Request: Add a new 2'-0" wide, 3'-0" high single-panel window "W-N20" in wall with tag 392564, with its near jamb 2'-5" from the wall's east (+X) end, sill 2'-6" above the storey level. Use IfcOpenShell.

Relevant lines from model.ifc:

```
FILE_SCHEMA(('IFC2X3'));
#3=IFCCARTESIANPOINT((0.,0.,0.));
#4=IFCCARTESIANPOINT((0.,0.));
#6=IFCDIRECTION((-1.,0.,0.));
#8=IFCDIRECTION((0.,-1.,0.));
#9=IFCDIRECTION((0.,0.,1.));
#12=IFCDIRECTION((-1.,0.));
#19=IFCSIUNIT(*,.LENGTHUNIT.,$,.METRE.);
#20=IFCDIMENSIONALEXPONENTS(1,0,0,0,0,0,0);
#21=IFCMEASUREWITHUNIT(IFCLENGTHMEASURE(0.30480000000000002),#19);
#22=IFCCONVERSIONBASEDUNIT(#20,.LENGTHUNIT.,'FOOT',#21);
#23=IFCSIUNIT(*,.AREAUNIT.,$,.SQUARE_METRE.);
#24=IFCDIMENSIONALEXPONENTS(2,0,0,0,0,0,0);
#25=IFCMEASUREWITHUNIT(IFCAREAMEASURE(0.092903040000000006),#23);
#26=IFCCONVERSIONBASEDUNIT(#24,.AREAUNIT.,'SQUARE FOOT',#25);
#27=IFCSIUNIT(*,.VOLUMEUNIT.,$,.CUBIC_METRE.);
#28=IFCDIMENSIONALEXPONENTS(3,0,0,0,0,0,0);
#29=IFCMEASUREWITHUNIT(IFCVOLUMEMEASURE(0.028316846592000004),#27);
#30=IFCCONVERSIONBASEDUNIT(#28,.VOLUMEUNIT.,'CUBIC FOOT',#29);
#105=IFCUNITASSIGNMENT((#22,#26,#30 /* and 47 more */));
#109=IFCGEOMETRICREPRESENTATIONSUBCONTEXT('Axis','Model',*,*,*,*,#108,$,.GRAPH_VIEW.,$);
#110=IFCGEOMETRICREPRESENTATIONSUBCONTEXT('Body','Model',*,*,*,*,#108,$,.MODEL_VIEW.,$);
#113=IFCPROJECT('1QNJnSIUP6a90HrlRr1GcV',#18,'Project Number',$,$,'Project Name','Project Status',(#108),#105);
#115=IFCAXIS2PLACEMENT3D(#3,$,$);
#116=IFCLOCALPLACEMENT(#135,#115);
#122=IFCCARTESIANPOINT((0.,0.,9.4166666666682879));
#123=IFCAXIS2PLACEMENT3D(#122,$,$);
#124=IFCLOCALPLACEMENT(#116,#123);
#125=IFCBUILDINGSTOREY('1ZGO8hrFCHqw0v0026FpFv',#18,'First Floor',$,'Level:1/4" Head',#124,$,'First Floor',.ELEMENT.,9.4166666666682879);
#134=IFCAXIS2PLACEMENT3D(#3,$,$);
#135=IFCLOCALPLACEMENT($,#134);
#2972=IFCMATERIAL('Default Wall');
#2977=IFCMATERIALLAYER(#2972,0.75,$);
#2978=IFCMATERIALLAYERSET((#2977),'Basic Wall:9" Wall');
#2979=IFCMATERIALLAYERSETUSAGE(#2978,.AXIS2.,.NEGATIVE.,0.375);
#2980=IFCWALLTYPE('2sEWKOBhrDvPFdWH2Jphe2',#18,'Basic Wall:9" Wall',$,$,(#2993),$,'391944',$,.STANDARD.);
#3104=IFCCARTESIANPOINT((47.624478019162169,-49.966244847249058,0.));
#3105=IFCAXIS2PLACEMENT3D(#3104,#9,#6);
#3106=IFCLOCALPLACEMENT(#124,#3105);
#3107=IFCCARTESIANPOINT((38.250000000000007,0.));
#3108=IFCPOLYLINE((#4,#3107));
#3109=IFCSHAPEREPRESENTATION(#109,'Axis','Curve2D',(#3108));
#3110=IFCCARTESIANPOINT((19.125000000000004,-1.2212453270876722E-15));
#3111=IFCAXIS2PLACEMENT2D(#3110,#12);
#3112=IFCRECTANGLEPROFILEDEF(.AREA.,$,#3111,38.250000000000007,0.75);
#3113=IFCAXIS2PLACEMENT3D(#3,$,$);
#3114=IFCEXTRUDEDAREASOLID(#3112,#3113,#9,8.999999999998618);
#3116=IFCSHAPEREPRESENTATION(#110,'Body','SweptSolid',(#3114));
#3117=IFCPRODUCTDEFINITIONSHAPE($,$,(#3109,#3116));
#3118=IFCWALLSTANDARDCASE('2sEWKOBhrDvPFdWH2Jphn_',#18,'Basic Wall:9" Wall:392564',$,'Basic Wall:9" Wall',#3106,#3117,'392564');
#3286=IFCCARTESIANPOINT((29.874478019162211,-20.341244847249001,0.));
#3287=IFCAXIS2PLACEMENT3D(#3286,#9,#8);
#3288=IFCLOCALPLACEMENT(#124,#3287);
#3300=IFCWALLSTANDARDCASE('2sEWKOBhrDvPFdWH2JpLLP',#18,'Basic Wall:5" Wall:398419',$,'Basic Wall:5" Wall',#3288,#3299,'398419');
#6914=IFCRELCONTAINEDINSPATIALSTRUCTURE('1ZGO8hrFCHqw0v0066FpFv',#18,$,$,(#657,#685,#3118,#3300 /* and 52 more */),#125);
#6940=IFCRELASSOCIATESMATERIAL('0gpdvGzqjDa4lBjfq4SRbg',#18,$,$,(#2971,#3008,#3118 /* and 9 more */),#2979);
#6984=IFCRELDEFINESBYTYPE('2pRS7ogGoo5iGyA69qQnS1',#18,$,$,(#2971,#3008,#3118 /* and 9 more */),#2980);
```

```python
import numpy as np
import ifcopenshell
import ifcopenshell.api.feature
import ifcopenshell.api.geometry
import ifcopenshell.api.root
import ifcopenshell.api.spatial
import ifcopenshell.api.type
import ifcopenshell.geom
import ifcopenshell.util.element
import ifcopenshell.util.placement
import ifcopenshell.util.representation
import ifcopenshell.util.shape
import ifcopenshell.util.unit

model = ifcopenshell.open("model.ifc")
unit_scale = ifcopenshell.util.unit.calculate_unit_scale(model)
settings = ifcopenshell.geom.settings()


def volume(element):
    """Net volume in cubic metres, openings subtracted."""
    shape = ifcopenshell.geom.create_shape(settings, element)
    return ifcopenshell.util.shape.get_volume(shape.geometry)


wall = model.by_id(3118)
storey = ifcopenshell.util.element.get_container(wall, ifc_class="IfcBuildingStorey")
context = ifcopenshell.util.representation.get_context(model, "Model", "Body", "MODEL_VIEW")
before = volume(wall)

width, height, from_end, sill = 0.6096, 0.9144, 0.7366, 0.762  # metres

# The wall runs along its own X axis, and the end named is its -X end.
wall_shape = ifcopenshell.geom.create_shape(settings, wall)
x, y, z = ifcopenshell.util.shape.get_vertices(wall_shape.geometry).T
start = x.min() + from_end
face, thickness = float(y.min()), float(y.max() - y.min())
wall_matrix = ifcopenshell.util.placement.get_local_placement(wall.ObjectPlacement)
level = ifcopenshell.util.placement.get_local_placement(storey.ObjectPlacement)[2, 3]


def in_wall(x, y):
    """Placement at x, y metres in the wall's axes, at sill height."""
    matrix = wall_matrix.copy()
    matrix[:, 3] = wall_matrix @ np.array([x / unit_scale, y / unit_scale, 0.0, 1.0])
    matrix[2, 3] = level + sill / unit_scale
    return matrix


# Opening: a box that overshoots both wall faces by 50 mm.
opening = ifcopenshell.api.root.create_entity(model, ifc_class="IfcOpeningElement")
box = ifcopenshell.api.geometry.add_wall_representation(
    model, context=context, length=width, height=height, thickness=thickness + 0.1
)
ifcopenshell.api.geometry.assign_representation(model, product=opening, representation=box)
ifcopenshell.api.geometry.edit_object_placement(model, product=opening, matrix=in_wall(start, face - 0.05), is_si=False)
ifcopenshell.api.feature.add_feature(model, feature=opening, element=wall)

window = ifcopenshell.api.root.create_entity(model, ifc_class="IfcWindow", name="W-N20")
window.OverallWidth, window.OverallHeight = width / unit_scale, height / unit_scale
body = ifcopenshell.api.geometry.add_window_representation(
    model,
    context=context,
    overall_width=window.OverallWidth,
    overall_height=window.OverallHeight,
    partition_type="SINGLE_PANEL",
)
ifcopenshell.api.geometry.assign_representation(model, product=window, representation=body)
ifcopenshell.api.spatial.assign_container(model, products=[window], relating_structure=storey)
fills = ifcopenshell.api.feature.add_filling(model, opening=opening, element=window)
fills.OwnerHistory = window.OwnerHistory  # required in IFC2X3

# IFC2X3 keeps the operation on the window style.
style = ifcopenshell.api.root.create_entity(model, ifc_class="IfcWindowStyle", name="W-N20")
style.OperationType, style.ConstructionType = "SINGLE_PANEL", "NOTDEFINED"
style.ParameterTakesPrecedence = style.Sizeable = False
ifcopenshell.api.type.assign_type(model, related_objects=[window], relating_type=style)

# Centre the window in the wall's thickness.
ifcopenshell.api.geometry.edit_object_placement(model, product=window, matrix=in_wall(start, face), is_si=False)
window_shape = ifcopenshell.geom.create_shape(settings, window)
depth = ifcopenshell.util.shape.get_vertices(window_shape.geometry)[:, 1]
offset = face + thickness / 2 - (depth.min() + depth.max()) / 2
ifcopenshell.api.geometry.edit_object_placement(model, product=window, matrix=in_wall(start, offset), is_si=False)

after = volume(wall)

print(f"wall volume {before:.3f} -> {after:.3f} m3")

model.write("model_v2.ifc")
```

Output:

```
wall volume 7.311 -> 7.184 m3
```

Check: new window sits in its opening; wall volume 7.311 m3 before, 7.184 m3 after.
